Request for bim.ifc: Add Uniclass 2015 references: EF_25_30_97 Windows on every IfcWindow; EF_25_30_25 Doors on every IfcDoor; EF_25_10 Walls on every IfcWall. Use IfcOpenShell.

First a look at what the model holds.

```python
import ifcopenshell

model = ifcopenshell.open("bim.ifc")
print(model.schema)
print("classifications:", [c.Name for c in model.by_type("IfcClassification")])
for ifc_class in ("IfcDoor", "IfcRoof", "IfcStair", "IfcWall", "IfcWindow"):
    print(ifc_class, len(model.by_type(ifc_class)))
```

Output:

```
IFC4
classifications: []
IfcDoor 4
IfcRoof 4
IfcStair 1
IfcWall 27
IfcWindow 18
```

```python
import ifcopenshell
import ifcopenshell.api.classification

model = ifcopenshell.open("bim.ifc")

system = ifcopenshell.api.classification.add_classification(model, classification="Uniclass 2015")

codes = {
    "IfcWindow": ("EF_25_30_97", "Windows"),
    "IfcDoor": ("EF_25_30_25", "Doors"),
    "IfcWall": ("EF_25_10", "Walls"),
}
for ifc_class, (code, name) in codes.items():
    products = model.by_type(ifc_class)
    ifcopenshell.api.classification.add_reference(
        model, products=products, classification=system, identification=code, name=name
    )
    print(code, len(products))

model.write("bim_rev.ifc")
```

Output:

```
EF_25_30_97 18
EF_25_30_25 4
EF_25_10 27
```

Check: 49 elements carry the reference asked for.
